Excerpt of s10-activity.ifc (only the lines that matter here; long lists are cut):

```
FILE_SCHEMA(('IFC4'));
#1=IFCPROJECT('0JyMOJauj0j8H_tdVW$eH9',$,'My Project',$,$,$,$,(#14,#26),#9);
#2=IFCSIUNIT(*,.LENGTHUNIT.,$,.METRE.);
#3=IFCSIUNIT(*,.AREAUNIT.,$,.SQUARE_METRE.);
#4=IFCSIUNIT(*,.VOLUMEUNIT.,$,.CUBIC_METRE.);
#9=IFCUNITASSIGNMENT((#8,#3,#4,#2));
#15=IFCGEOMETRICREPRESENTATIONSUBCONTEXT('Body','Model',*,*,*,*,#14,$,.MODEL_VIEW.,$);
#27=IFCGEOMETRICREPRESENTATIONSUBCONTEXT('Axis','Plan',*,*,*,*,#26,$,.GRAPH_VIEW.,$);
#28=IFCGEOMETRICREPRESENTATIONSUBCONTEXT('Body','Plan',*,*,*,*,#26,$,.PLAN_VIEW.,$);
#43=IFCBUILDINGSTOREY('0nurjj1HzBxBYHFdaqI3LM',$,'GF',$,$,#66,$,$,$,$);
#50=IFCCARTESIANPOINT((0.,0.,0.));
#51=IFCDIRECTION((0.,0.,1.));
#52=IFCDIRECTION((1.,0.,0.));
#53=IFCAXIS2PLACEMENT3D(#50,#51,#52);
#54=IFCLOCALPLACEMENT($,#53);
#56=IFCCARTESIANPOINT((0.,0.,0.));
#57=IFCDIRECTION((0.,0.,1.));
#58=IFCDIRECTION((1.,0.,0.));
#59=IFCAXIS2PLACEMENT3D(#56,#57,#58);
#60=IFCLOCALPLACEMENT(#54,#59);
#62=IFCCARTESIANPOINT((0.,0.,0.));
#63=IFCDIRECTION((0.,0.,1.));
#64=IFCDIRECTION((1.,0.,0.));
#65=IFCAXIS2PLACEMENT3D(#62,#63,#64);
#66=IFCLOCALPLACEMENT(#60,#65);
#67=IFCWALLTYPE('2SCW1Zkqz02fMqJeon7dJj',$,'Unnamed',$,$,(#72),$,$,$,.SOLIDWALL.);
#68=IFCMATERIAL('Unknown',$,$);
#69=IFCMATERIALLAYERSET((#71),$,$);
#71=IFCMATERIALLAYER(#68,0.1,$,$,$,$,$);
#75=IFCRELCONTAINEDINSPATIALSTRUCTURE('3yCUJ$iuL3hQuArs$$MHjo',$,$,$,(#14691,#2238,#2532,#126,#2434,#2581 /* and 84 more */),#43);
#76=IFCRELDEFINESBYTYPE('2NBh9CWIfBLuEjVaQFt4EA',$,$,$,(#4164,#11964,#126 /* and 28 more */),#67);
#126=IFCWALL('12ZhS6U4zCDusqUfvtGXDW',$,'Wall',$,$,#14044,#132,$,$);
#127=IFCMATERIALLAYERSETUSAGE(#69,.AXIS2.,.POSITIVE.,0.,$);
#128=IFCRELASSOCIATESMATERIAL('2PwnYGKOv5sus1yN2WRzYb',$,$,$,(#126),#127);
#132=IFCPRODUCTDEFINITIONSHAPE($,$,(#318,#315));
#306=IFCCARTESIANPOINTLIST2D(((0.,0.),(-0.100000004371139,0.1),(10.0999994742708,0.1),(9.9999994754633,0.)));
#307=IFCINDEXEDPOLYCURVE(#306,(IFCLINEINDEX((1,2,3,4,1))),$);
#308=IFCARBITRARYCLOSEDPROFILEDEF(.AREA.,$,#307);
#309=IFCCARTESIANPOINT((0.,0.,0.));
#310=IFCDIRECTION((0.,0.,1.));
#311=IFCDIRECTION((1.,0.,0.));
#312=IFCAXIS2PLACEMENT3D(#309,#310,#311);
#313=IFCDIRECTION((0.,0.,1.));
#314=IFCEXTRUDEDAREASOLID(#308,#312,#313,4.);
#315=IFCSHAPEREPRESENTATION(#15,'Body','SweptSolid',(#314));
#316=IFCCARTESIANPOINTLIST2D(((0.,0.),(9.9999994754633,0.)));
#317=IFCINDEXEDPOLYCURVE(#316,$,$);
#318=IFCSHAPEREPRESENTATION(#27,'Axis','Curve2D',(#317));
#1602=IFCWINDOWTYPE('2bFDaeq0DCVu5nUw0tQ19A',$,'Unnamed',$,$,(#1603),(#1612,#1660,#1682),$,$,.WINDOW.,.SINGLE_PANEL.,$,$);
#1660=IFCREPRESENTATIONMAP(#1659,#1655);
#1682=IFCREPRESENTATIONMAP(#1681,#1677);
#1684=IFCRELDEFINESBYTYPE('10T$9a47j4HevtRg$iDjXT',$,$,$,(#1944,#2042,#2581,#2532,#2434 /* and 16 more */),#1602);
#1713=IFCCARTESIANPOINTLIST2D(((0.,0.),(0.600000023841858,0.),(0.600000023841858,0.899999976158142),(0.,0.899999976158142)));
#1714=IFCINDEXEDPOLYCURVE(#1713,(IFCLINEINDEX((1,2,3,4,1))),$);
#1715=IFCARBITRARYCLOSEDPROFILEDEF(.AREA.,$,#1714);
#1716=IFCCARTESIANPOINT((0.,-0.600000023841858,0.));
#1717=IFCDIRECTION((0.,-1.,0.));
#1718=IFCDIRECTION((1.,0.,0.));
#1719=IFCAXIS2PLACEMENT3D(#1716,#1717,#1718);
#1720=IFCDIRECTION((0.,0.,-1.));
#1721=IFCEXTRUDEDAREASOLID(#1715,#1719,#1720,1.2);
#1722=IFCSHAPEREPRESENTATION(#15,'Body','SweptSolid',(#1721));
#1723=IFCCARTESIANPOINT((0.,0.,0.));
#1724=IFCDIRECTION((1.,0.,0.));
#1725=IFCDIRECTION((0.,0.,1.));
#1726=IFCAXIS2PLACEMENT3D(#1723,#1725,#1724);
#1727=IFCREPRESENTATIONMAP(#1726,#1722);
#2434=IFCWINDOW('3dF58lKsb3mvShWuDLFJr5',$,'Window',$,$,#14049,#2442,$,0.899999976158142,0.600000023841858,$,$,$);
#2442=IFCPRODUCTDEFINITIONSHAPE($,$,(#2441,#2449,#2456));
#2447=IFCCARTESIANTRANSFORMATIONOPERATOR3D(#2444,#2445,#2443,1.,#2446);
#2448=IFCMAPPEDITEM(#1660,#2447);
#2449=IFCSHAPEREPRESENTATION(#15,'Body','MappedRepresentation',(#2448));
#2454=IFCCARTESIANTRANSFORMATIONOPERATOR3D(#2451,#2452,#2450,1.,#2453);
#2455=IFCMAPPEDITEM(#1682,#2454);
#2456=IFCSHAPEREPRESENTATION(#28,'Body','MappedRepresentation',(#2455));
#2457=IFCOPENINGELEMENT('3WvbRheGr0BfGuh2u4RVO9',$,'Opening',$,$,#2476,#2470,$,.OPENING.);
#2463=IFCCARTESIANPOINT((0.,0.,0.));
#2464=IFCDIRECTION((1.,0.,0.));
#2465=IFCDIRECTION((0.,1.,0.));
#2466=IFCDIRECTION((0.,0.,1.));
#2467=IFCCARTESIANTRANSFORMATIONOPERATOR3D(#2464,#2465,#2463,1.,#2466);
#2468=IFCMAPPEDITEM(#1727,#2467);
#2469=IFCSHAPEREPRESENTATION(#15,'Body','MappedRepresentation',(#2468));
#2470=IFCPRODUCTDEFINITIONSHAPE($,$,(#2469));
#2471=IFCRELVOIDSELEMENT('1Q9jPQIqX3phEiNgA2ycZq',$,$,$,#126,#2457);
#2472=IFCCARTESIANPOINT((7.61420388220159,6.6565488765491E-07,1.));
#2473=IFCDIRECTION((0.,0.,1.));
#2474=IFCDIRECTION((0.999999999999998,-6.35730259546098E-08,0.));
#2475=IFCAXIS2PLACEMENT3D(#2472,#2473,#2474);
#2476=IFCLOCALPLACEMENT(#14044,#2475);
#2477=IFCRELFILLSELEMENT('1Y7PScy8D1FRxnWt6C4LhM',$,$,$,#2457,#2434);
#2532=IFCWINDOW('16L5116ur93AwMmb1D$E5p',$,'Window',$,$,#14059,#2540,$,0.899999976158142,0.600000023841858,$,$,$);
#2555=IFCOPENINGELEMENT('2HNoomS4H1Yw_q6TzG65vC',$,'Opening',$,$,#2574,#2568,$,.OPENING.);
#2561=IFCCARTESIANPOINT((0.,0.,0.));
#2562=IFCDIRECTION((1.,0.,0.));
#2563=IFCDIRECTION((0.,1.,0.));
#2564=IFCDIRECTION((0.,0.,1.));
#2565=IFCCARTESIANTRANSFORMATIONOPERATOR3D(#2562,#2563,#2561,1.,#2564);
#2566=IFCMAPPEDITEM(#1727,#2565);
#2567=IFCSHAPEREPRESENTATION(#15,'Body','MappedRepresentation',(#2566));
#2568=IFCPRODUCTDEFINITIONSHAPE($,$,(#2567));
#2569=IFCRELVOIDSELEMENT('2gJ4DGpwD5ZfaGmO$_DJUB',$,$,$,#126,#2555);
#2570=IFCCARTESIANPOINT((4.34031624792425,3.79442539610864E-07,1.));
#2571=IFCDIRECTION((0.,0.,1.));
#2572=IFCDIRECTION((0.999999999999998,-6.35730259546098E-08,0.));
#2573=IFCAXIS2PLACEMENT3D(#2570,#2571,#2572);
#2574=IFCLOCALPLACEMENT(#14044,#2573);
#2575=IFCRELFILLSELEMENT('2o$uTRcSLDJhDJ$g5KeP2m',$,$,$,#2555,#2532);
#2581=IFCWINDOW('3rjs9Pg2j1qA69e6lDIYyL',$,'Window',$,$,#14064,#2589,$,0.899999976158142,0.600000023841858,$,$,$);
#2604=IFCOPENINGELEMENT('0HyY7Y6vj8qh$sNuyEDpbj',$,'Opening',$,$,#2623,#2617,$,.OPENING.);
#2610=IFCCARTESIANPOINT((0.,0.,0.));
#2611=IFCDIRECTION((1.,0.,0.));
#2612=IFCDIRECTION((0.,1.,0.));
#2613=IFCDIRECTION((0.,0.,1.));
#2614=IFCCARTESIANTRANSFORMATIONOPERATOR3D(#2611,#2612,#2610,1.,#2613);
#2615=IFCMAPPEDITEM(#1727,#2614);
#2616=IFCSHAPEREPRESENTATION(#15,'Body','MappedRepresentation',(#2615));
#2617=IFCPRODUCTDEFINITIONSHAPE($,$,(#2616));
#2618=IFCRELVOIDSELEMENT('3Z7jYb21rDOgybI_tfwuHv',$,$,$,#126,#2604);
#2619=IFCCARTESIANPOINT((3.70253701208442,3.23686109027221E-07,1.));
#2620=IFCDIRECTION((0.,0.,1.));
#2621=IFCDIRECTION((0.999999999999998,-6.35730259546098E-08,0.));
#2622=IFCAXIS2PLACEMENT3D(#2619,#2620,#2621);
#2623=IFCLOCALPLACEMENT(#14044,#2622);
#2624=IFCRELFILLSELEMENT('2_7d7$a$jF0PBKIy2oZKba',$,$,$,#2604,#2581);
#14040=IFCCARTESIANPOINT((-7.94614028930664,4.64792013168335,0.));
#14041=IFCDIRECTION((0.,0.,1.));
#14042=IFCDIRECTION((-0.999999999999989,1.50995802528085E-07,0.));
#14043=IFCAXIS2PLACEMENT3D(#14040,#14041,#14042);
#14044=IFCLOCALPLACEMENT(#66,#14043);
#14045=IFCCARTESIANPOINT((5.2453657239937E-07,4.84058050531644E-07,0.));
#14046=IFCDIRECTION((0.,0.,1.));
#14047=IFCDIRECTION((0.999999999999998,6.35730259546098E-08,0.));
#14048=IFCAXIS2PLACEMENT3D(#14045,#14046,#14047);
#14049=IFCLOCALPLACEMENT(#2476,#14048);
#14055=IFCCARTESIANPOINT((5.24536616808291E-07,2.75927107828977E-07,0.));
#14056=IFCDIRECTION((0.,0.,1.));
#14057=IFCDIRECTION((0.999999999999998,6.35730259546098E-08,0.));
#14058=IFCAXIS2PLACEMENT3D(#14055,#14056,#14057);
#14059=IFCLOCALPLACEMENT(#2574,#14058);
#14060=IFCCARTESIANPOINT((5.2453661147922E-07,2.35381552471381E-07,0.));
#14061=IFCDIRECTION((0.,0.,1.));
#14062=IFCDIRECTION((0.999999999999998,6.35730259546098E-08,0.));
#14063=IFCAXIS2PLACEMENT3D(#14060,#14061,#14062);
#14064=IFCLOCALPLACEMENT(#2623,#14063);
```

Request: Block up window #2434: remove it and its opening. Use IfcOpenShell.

```python
import ifcopenshell
import ifcopenshell.api.feature
import ifcopenshell.api.root
import ifcopenshell.geom
import ifcopenshell.util.shape

model = ifcopenshell.open("s10-activity.ifc")
settings = ifcopenshell.geom.settings()


def volume(element):
    """Net volume in cubic metres, openings subtracted."""
    shape = ifcopenshell.geom.create_shape(settings, element)
    return ifcopenshell.util.shape.get_volume(shape.geometry)


window = model.by_id(2434)
opening = window.FillsVoids[0].RelatingOpeningElement
wall = opening.VoidsElements[0].RelatingBuildingElement
before = volume(wall)

ifcopenshell.api.root.remove_product(model, product=window)
ifcopenshell.api.feature.remove_feature(model, feature=opening)

after = volume(wall)

print(f"wall volume {before:.3f} -> {after:.3f} m3")

model.write("s10-activity_v2.ifc")
```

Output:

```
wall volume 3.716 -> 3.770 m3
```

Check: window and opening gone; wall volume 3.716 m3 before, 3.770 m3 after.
